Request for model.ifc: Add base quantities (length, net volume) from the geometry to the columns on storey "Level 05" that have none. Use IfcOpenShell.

First a look at what the model holds.

```python
import ifcopenshell
import ifcopenshell.util.element
import ifcopenshell.util.unit

model = ifcopenshell.open("model.ifc")
print(model.schema)
for unit_type in ("LENGTHUNIT", "AREAUNIT", "VOLUMEUNIT"):
    print(unit_type, ifcopenshell.util.unit.calculate_unit_scale(model, unit_type))
storey = next(s for s in model.by_type("IfcBuildingStorey") if s.Name == "Level 05")
columns = [e for e in ifcopenshell.util.element.get_decomposition(storey) if e.is_a("IfcColumn")]
for e in sorted(columns, key=lambda e: e.id()):
    print(e.id(), e.is_a(), e.Name, list(ifcopenshell.util.element.get_psets(e, qtos_only=True)), sep=" | ")
```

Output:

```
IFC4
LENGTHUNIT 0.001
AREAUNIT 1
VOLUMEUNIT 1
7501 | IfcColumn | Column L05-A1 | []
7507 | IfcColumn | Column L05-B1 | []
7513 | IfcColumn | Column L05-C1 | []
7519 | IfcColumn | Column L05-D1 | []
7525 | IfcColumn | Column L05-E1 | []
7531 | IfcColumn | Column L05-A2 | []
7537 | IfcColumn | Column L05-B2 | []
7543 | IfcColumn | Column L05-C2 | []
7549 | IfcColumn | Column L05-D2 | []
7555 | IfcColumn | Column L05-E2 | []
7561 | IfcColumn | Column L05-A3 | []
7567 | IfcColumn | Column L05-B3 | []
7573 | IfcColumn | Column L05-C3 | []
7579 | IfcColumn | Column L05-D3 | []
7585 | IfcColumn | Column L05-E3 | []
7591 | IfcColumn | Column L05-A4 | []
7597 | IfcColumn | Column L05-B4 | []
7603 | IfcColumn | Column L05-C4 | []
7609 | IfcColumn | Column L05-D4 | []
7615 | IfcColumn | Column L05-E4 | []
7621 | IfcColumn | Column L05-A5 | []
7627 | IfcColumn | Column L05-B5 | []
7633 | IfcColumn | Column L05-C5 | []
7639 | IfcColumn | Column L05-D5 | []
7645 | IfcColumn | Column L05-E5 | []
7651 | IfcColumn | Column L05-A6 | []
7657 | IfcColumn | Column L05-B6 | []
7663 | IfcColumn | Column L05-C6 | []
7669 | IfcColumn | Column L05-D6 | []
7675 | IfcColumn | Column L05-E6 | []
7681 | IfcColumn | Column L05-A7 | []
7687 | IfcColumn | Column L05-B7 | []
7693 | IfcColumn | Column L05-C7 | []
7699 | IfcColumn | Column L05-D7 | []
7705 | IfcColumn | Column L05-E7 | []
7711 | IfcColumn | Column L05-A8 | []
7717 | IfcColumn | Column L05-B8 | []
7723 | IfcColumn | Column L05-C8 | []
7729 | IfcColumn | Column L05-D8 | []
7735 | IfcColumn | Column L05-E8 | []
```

```python
import ifcopenshell
import ifcopenshell.api.pset
import ifcopenshell.geom
import ifcopenshell.util.element
import ifcopenshell.util.shape
import ifcopenshell.util.unit

model = ifcopenshell.open("model.ifc")
unit_scale = ifcopenshell.util.unit.calculate_unit_scale(model)
volume_scale = ifcopenshell.util.unit.calculate_unit_scale(model, "VOLUMEUNIT")
settings = ifcopenshell.geom.settings()

storey = next(s for s in model.by_type("IfcBuildingStorey") if s.Name == "Level 05")
columns = [e for e in ifcopenshell.util.element.get_decomposition(storey) if e.is_a("IfcColumn")]

for e in sorted(columns, key=lambda e: e.id()):
    if ifcopenshell.util.element.get_psets(e, qtos_only=True, should_inherit=False):
        continue
    # Geometry comes back in metres, in the element's own axes.
    shape = ifcopenshell.geom.create_shape(settings, e)
    values = {
        "Length": ifcopenshell.util.shape.get_z(shape.geometry) / unit_scale,
        "NetVolume": ifcopenshell.util.shape.get_volume(shape.geometry) / volume_scale,
    }
    qto = ifcopenshell.api.pset.add_qto(model, product=e, name="Qto_ColumnBaseQuantities")
    ifcopenshell.api.pset.edit_qto(model, qto=qto, properties=values)
    print(e.id(), {k: round(v, 3) for k, v in values.items()})

model.write("model-out.ifc")
```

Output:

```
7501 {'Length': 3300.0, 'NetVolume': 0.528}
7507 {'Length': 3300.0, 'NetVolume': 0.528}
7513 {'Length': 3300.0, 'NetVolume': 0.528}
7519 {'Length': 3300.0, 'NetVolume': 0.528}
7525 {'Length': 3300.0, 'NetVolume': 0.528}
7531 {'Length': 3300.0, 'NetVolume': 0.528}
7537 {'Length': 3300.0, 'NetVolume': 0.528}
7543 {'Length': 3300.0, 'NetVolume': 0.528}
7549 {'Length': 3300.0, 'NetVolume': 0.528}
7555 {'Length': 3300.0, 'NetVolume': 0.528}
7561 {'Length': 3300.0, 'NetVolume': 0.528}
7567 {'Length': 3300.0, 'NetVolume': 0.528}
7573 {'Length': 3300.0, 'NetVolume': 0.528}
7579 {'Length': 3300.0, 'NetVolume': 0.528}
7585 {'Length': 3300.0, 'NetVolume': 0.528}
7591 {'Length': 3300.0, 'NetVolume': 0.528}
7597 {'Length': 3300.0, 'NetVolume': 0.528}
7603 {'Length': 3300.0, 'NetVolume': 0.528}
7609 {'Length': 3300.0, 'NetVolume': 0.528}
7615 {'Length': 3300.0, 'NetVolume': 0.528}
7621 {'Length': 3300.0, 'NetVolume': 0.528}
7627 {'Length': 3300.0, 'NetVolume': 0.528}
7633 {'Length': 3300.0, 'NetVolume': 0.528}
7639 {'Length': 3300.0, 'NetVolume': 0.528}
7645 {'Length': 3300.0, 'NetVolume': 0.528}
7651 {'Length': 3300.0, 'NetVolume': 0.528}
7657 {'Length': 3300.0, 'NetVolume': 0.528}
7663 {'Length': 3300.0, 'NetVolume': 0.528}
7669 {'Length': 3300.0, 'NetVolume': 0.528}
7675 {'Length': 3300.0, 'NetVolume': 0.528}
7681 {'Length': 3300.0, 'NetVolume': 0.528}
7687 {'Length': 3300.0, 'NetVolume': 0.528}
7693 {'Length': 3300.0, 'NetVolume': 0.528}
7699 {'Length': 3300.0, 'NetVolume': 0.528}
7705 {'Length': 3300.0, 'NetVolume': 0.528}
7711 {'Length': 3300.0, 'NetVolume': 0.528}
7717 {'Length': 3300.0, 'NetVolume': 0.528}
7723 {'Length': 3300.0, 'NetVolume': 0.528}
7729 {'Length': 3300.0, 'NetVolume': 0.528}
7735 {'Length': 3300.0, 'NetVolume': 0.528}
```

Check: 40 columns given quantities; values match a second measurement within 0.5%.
